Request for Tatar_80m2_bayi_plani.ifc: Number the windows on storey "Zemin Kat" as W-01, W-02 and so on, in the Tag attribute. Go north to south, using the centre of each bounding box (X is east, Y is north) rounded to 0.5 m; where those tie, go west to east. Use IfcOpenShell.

First a look at what the model holds.

```python
import ifcopenshell
import ifcopenshell.util.element
import ifcopenshell.util.placement

model = ifcopenshell.open("Tatar_80m2_bayi_plani.ifc")
print(model.schema)
storey = next(s for s in model.by_type("IfcBuildingStorey") if s.Name == "Zemin Kat")
windows = [e for e in ifcopenshell.util.element.get_decomposition(storey) if e.is_a("IfcWindow")]
for e in sorted(windows, key=lambda e: e.id()):
    origin = ifcopenshell.util.placement.get_local_placement(e.ObjectPlacement)[:3, 3]
    print(e.id(), e.Tag, e.Name, origin.round(2) + 0.0, sep=" | ")
```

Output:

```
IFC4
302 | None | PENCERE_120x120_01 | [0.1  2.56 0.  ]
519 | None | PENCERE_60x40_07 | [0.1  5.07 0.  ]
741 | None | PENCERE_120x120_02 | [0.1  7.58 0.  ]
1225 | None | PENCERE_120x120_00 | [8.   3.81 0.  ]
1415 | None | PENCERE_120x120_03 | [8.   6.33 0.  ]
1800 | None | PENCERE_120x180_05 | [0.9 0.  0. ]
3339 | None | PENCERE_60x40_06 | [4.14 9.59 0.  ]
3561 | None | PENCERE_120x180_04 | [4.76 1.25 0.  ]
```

```python
import ifcopenshell
import ifcopenshell.geom
import ifcopenshell.util.element
import ifcopenshell.util.shape

model = ifcopenshell.open("Tatar_80m2_bayi_plani.ifc")
settings = ifcopenshell.geom.settings()
settings.set("use-world-coords", True)


def centre(element):
    shape = ifcopenshell.geom.create_shape(settings, element)
    return ifcopenshell.util.shape.get_bbox_centroid(shape.geometry)


storey = next(s for s in model.by_type("IfcBuildingStorey") if s.Name == "Zemin Kat")
windows = [e for e in ifcopenshell.util.element.get_decomposition(storey) if e.is_a("IfcWindow")]

# Insertion points can sit at a corner or the storey origin, so sort by the geometry (in metres).
centres = {e: centre(e) for e in windows}
windows.sort(key=lambda e: (-round(centres[e][1] / 0.5), centres[e][0]))

for i, e in enumerate(windows, start=1):
    number = f"W-{i:02d}"
    e.Tag = number
    print(e.id(), number)

model.write("Tatar_80m2_bayi_plani_updated.ifc")
```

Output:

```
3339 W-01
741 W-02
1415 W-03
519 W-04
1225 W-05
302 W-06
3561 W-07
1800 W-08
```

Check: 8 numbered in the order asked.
